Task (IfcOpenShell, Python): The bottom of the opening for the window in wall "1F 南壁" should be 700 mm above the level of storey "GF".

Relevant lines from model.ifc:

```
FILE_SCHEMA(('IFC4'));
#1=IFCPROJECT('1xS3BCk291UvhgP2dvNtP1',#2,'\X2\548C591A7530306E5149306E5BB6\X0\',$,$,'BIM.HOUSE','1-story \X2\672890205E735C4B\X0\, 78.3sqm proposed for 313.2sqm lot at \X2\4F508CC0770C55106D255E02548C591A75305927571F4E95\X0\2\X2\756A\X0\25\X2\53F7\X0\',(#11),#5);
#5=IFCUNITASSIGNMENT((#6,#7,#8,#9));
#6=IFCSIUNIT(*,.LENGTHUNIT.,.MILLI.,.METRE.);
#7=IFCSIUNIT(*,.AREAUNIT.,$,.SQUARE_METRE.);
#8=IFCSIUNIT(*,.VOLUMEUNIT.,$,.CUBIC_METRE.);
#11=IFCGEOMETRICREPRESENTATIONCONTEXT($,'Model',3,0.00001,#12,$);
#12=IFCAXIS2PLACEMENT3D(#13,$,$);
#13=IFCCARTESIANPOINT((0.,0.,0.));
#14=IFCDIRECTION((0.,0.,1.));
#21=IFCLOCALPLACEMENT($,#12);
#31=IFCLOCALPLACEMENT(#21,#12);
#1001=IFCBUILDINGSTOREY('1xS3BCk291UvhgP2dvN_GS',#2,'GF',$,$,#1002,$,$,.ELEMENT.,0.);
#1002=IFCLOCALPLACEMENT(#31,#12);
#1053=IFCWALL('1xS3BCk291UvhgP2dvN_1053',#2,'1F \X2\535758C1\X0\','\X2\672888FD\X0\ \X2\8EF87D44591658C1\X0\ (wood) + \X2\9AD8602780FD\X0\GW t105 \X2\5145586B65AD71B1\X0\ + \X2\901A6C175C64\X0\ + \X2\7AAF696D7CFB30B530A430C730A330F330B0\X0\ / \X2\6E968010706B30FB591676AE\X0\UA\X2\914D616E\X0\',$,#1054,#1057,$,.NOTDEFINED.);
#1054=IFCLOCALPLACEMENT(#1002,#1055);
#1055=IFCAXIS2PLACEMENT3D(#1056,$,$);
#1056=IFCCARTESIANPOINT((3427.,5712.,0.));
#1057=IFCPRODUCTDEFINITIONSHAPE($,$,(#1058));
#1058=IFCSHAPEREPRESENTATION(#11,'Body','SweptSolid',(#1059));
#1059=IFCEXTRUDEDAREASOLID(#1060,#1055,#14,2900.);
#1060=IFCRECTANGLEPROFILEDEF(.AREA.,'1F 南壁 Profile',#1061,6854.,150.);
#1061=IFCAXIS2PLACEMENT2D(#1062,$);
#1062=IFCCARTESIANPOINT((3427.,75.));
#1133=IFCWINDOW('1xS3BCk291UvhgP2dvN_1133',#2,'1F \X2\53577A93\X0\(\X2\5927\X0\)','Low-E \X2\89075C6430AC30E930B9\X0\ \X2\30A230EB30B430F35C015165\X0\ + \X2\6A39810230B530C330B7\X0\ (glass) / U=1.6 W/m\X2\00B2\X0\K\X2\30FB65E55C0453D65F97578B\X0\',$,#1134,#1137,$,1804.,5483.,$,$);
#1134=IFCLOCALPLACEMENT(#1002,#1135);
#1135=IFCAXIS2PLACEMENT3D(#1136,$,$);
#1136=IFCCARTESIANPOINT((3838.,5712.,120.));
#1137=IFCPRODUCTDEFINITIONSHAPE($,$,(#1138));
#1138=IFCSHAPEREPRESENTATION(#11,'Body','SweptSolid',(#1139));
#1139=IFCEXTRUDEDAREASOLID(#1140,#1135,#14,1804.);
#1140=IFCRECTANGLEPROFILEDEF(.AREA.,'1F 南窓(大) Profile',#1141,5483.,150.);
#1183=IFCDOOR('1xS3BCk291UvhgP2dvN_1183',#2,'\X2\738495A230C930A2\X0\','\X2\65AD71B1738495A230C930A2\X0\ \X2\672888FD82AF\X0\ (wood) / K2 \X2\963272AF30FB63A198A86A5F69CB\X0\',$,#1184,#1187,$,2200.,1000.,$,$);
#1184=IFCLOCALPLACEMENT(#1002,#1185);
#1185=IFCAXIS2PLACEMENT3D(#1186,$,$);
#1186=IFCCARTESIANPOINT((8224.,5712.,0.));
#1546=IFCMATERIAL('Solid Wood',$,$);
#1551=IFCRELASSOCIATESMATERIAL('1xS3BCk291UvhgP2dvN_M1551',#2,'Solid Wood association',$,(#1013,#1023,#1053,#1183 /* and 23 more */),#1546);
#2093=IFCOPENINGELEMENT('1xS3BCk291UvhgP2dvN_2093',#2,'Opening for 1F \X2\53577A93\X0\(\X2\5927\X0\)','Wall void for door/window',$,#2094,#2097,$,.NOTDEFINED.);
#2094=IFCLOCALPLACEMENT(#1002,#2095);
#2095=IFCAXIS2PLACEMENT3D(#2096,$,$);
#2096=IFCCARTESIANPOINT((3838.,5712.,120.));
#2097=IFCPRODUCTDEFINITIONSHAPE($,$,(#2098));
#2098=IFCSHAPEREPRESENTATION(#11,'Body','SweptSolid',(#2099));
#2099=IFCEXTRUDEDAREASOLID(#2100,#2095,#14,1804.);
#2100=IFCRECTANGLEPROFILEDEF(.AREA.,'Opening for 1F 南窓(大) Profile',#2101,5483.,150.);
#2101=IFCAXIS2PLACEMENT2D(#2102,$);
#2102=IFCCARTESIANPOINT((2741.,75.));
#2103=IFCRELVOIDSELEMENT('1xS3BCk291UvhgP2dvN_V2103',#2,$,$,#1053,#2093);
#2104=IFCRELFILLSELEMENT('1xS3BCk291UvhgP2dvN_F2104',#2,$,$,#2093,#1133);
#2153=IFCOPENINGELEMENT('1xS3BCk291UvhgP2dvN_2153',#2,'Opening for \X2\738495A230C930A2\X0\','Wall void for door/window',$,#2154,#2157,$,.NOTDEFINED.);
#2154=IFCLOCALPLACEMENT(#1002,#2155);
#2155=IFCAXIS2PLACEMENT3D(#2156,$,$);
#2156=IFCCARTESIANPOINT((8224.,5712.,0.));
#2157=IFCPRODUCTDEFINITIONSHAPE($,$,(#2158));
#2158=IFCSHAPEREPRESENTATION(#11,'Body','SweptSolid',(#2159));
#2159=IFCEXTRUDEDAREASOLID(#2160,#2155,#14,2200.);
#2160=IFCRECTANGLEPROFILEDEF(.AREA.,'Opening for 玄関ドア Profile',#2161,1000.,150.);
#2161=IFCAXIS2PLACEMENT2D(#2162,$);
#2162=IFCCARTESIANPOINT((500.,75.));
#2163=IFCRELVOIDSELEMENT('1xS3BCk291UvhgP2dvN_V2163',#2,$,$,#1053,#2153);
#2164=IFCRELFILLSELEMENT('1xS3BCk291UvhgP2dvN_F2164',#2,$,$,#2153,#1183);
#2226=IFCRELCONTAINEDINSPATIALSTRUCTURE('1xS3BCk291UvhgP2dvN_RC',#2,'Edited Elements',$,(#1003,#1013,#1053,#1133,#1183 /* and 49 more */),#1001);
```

```python
import numpy as np
import ifcopenshell
import ifcopenshell.api.geometry
import ifcopenshell.geom
import ifcopenshell.util.element
import ifcopenshell.util.placement
import ifcopenshell.util.shape
import ifcopenshell.util.unit

model = ifcopenshell.open("model.ifc")
unit_scale = ifcopenshell.util.unit.calculate_unit_scale(model)

window = model.by_guid("1xS3BCk291UvhgP2dvN_1133")
opening = window.FillsVoids[0].RelatingOpeningElement
storey = ifcopenshell.util.element.get_container(window, ifc_class="IfcBuildingStorey")
level = ifcopenshell.util.placement.get_local_placement(storey.ObjectPlacement)[2, 3]

# The opening's origin need not be at the sill, so measure its lowest point.
shape = ifcopenshell.geom.create_shape(ifcopenshell.geom.settings(), opening)
bottom = ifcopenshell.util.shape.get_shape_bottom_elevation(shape, shape.geometry) / unit_scale
dz = level + 700.0 - bottom

shift = np.array([0.0, 0.0, dz])
# The window is not placed relative to its opening, so move both.
for product in (opening, window):
    matrix = ifcopenshell.util.placement.get_local_placement(product.ObjectPlacement)
    matrix[:3, 3] += shift
    ifcopenshell.api.geometry.edit_object_placement(model, product=product, matrix=matrix, is_si=False)

print(f"moved by {dz * unit_scale:+.3f} m")

model.write("model-out.ifc")
```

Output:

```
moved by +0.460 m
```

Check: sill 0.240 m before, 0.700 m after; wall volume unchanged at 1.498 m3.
